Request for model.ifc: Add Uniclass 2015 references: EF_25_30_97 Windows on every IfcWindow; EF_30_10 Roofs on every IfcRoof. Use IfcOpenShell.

First a look at what the model holds.

```python
import ifcopenshell

model = ifcopenshell.open("model.ifc")
print(model.schema)
print("classifications:", [c.Name for c in model.by_type("IfcClassification")])
for ifc_class in ("IfcDoor", "IfcRoof", "IfcStair", "IfcWall", "IfcWindow"):
    print(ifc_class, len(model.by_type(ifc_class)))
```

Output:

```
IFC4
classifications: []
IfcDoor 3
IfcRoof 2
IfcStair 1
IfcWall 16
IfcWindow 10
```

```python
import ifcopenshell
import ifcopenshell.api.classification

model = ifcopenshell.open("model.ifc")

system = ifcopenshell.api.classification.add_classification(model, classification="Uniclass 2015")

codes = {
    "IfcWindow": ("EF_25_30_97", "Windows"),
    "IfcRoof": ("EF_30_10", "Roofs"),
}
for ifc_class, (code, name) in codes.items():
    products = model.by_type(ifc_class)
    ifcopenshell.api.classification.add_reference(
        model, products=products, classification=system, identification=code, name=name
    )
    print(code, len(products))

model.write("model_updated.ifc")
```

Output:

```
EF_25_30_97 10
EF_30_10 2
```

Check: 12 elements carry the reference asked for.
